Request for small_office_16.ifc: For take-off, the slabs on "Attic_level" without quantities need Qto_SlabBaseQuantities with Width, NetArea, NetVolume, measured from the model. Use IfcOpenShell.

First a look at what the model holds.

```python
import ifcopenshell
import ifcopenshell.util.element
import ifcopenshell.util.unit

model = ifcopenshell.open("small_office_16.ifc")
print(model.schema)
for unit_type in ("LENGTHUNIT", "AREAUNIT", "VOLUMEUNIT"):
    print(unit_type, ifcopenshell.util.unit.calculate_unit_scale(model, unit_type))
storey = next(s for s in model.by_type("IfcBuildingStorey") if s.Name == "Attic_level")
slabs = [e for e in ifcopenshell.util.element.get_decomposition(storey) if e.is_a("IfcSlab")]
for e in sorted(slabs, key=lambda e: e.id()):
    print(e.id(), e.is_a(), e.Name, list(ifcopenshell.util.element.get_psets(e, qtos_only=True)), sep=" | ")
```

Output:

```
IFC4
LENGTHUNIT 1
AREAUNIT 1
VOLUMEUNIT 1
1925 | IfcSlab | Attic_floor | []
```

```python
import ifcopenshell
import ifcopenshell.api.pset
import ifcopenshell.geom
import ifcopenshell.util.element
import ifcopenshell.util.shape
import ifcopenshell.util.unit

model = ifcopenshell.open("small_office_16.ifc")
unit_scale = ifcopenshell.util.unit.calculate_unit_scale(model)
area_scale = ifcopenshell.util.unit.calculate_unit_scale(model, "AREAUNIT")
volume_scale = ifcopenshell.util.unit.calculate_unit_scale(model, "VOLUMEUNIT")
settings = ifcopenshell.geom.settings()

storey = next(s for s in model.by_type("IfcBuildingStorey") if s.Name == "Attic_level")
slabs = [e for e in ifcopenshell.util.element.get_decomposition(storey) if e.is_a("IfcSlab")]

for e in sorted(slabs, key=lambda e: e.id()):
    if ifcopenshell.util.element.get_psets(e, qtos_only=True, should_inherit=False):
        continue
    # Geometry comes back in metres, in the element's own axes.
    shape = ifcopenshell.geom.create_shape(settings, e)
    values = {
        "Width": ifcopenshell.util.shape.get_z(shape.geometry) / unit_scale,
        "NetArea": ifcopenshell.util.shape.get_footprint_area(shape.geometry) / area_scale,
        "NetVolume": ifcopenshell.util.shape.get_volume(shape.geometry) / volume_scale,
    }
    qto = ifcopenshell.api.pset.add_qto(model, product=e, name="Qto_SlabBaseQuantities")
    ifcopenshell.api.pset.edit_qto(model, qto=qto, properties=values)
    print(e.id(), {k: round(v, 3) for k, v in values.items()})

model.write("small_office_16_v2.ifc")
```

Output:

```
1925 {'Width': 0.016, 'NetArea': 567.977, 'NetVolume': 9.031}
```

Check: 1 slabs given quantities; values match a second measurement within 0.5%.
